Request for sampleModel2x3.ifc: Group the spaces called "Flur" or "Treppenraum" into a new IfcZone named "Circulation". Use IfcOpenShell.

First a look at what the model holds.

```python
import ifcopenshell

model = ifcopenshell.open("sampleModel2x3.ifc")
print(model.schema)
seen = {}
for space in model.by_type("IfcSpace"):
    seen[space.LongName] = seen.get(space.LongName, 0) + 1
for name, count in sorted(seen.items(), key=str):
    print(count, "x", name)
print("zones:", [z.Name for z in model.by_type("IfcZone")][:20])
```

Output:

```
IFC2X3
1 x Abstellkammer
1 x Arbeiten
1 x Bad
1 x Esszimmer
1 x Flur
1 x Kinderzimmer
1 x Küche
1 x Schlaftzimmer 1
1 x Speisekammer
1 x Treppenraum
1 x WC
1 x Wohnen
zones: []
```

```python
import ifcopenshell
import ifcopenshell.api.group
import ifcopenshell.api.root

model = ifcopenshell.open("sampleModel2x3.ifc")

names = {"Flur", "Treppenraum"}
spaces = [s for s in model.by_type("IfcSpace") if s.LongName in names]

zone = ifcopenshell.api.root.create_entity(model, ifc_class="IfcZone", name="Circulation")
ifcopenshell.api.group.assign_group(model, products=spaces, group=zone)
print(len(spaces), "spaces in", zone.Name)

model.write("sampleModel2x3_rev.ifc")
```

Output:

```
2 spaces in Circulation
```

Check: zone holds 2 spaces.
